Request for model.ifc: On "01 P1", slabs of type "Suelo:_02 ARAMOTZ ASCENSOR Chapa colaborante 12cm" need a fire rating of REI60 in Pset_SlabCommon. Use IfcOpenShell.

First a look at what the model holds.

```python
import ifcopenshell
import ifcopenshell.util.element

model = ifcopenshell.open("model.ifc")
print(model.schema)
storey = next(s for s in model.by_type("IfcBuildingStorey") if s.Name == "01 P1")
slabs = [e for e in ifcopenshell.util.element.get_decomposition(storey) if e.is_a("IfcSlab")]
seen = {}
for e in slabs:
    element_type = ifcopenshell.util.element.get_type(e)
    key = (element_type.Name if element_type != e and element_type else None, ifcopenshell.util.element.get_pset(e, "Pset_SlabCommon", "FireRating"))
    seen[key] = seen.get(key, 0) + 1
for (name, value), count in sorted(seen.items(), key=str):
    print(count, "x", name, "|", value)
```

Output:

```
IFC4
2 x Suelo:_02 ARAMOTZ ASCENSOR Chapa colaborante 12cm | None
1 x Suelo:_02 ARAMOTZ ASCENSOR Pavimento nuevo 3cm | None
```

```python
import ifcopenshell
import ifcopenshell.api.pset
import ifcopenshell.util.element

model = ifcopenshell.open("model.ifc")

storey = next(s for s in model.by_type("IfcBuildingStorey") if s.Name == "01 P1")
slabs = [e for e in ifcopenshell.util.element.get_decomposition(storey) if e.is_a("IfcSlab")]

count = 0
for e in slabs:
    element_type = ifcopenshell.util.element.get_type(e)
    if element_type in (None, e) or element_type.Name != "Suelo:_02 ARAMOTZ ASCENSOR Chapa colaborante 12cm":
        continue
    # add_pset returns the element's existing set when there is one.
    pset = ifcopenshell.api.pset.add_pset(model, product=e, name="Pset_SlabCommon")
    ifcopenshell.api.pset.edit_pset(model, pset=pset, properties={"FireRating": "REI60"})
    count += 1

print(count, "slabs updated")

model.write("model-out.ifc")
```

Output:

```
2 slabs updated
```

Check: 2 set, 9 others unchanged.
